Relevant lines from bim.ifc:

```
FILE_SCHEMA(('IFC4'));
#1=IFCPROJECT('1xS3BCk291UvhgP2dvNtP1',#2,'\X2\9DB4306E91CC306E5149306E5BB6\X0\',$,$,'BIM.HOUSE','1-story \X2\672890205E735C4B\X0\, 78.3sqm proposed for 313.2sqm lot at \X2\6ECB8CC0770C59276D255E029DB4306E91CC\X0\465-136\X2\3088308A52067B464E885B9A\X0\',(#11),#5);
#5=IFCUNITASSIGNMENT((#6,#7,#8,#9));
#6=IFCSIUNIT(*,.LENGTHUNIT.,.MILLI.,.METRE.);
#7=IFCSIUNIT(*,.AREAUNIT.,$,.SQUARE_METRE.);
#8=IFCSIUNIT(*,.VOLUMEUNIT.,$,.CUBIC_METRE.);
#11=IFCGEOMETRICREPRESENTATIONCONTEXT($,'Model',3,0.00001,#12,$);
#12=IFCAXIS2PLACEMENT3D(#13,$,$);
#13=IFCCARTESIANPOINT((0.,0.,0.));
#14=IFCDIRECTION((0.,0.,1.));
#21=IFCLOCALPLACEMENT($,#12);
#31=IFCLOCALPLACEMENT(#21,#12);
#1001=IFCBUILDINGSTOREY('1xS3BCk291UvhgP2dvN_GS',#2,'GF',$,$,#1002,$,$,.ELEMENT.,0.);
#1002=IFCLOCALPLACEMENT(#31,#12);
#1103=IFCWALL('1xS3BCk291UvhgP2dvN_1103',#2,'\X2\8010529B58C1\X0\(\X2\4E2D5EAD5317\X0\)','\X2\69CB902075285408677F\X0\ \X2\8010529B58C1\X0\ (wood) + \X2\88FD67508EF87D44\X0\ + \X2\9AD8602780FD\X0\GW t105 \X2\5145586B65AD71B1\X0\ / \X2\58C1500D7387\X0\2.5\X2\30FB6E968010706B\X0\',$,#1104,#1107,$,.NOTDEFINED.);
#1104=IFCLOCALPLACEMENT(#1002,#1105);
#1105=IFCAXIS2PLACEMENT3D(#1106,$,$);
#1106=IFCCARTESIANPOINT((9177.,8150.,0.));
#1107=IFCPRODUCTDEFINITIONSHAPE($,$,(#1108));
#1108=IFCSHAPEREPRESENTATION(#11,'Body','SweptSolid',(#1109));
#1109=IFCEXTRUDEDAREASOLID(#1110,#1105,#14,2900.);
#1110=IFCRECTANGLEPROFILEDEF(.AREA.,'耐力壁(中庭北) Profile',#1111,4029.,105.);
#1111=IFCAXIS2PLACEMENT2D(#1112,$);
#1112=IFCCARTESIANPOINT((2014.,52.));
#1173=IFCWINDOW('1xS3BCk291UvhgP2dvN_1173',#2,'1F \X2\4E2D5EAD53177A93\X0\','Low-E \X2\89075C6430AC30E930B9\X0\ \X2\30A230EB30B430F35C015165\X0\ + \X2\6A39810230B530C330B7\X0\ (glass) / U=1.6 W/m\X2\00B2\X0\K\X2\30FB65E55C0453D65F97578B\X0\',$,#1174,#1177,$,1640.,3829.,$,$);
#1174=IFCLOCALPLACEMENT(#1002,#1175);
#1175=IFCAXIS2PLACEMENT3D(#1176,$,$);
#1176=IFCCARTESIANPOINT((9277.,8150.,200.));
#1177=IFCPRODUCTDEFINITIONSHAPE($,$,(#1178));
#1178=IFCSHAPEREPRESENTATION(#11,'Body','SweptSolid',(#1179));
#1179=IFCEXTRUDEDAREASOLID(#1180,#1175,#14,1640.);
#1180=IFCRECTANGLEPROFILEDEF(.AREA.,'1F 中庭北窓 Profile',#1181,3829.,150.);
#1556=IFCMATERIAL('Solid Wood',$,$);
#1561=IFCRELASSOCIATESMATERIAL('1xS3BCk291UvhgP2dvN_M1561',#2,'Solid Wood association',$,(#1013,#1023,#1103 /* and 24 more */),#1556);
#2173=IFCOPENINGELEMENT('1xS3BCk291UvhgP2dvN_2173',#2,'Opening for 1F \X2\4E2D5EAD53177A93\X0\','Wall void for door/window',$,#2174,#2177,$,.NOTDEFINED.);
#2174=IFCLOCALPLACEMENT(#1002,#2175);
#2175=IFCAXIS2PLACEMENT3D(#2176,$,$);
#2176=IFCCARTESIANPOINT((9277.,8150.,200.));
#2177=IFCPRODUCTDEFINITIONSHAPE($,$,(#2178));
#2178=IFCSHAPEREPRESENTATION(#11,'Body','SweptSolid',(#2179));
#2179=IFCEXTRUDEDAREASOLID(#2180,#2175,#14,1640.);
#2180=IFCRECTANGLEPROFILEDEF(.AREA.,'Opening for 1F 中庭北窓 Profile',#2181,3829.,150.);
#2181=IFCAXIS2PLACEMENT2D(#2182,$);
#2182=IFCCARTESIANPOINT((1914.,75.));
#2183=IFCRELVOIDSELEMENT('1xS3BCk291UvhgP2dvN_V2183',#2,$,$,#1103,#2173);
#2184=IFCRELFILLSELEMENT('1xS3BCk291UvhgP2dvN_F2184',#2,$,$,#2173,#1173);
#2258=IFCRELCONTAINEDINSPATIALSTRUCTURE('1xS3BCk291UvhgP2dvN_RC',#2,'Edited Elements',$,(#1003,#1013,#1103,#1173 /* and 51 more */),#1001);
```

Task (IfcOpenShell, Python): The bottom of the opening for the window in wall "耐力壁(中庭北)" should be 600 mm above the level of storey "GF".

```python
import numpy as np
import ifcopenshell
import ifcopenshell.api.geometry
import ifcopenshell.geom
import ifcopenshell.util.element
import ifcopenshell.util.placement
import ifcopenshell.util.shape
import ifcopenshell.util.unit

model = ifcopenshell.open("bim.ifc")
unit_scale = ifcopenshell.util.unit.calculate_unit_scale(model)

window = model.by_guid("1xS3BCk291UvhgP2dvN_1173")
opening = window.FillsVoids[0].RelatingOpeningElement
storey = ifcopenshell.util.element.get_container(window, ifc_class="IfcBuildingStorey")
level = ifcopenshell.util.placement.get_local_placement(storey.ObjectPlacement)[2, 3]

# The opening's origin need not be at the sill, so measure its lowest point.
shape = ifcopenshell.geom.create_shape(ifcopenshell.geom.settings(), opening)
bottom = ifcopenshell.util.shape.get_shape_bottom_elevation(shape, shape.geometry) / unit_scale
dz = level + 600.0 - bottom

shift = np.array([0.0, 0.0, dz])
# The window is not placed relative to its opening, so move both.
for product in (opening, window):
    matrix = ifcopenshell.util.placement.get_local_placement(product.ObjectPlacement)
    matrix[:3, 3] += shift
    ifcopenshell.api.geometry.edit_object_placement(model, product=product, matrix=matrix, is_si=False)

print(f"moved by {dz * unit_scale:+.3f} m")

model.write("bim_updated.ifc")
```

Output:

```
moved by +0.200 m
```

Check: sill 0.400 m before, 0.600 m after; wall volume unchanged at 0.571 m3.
